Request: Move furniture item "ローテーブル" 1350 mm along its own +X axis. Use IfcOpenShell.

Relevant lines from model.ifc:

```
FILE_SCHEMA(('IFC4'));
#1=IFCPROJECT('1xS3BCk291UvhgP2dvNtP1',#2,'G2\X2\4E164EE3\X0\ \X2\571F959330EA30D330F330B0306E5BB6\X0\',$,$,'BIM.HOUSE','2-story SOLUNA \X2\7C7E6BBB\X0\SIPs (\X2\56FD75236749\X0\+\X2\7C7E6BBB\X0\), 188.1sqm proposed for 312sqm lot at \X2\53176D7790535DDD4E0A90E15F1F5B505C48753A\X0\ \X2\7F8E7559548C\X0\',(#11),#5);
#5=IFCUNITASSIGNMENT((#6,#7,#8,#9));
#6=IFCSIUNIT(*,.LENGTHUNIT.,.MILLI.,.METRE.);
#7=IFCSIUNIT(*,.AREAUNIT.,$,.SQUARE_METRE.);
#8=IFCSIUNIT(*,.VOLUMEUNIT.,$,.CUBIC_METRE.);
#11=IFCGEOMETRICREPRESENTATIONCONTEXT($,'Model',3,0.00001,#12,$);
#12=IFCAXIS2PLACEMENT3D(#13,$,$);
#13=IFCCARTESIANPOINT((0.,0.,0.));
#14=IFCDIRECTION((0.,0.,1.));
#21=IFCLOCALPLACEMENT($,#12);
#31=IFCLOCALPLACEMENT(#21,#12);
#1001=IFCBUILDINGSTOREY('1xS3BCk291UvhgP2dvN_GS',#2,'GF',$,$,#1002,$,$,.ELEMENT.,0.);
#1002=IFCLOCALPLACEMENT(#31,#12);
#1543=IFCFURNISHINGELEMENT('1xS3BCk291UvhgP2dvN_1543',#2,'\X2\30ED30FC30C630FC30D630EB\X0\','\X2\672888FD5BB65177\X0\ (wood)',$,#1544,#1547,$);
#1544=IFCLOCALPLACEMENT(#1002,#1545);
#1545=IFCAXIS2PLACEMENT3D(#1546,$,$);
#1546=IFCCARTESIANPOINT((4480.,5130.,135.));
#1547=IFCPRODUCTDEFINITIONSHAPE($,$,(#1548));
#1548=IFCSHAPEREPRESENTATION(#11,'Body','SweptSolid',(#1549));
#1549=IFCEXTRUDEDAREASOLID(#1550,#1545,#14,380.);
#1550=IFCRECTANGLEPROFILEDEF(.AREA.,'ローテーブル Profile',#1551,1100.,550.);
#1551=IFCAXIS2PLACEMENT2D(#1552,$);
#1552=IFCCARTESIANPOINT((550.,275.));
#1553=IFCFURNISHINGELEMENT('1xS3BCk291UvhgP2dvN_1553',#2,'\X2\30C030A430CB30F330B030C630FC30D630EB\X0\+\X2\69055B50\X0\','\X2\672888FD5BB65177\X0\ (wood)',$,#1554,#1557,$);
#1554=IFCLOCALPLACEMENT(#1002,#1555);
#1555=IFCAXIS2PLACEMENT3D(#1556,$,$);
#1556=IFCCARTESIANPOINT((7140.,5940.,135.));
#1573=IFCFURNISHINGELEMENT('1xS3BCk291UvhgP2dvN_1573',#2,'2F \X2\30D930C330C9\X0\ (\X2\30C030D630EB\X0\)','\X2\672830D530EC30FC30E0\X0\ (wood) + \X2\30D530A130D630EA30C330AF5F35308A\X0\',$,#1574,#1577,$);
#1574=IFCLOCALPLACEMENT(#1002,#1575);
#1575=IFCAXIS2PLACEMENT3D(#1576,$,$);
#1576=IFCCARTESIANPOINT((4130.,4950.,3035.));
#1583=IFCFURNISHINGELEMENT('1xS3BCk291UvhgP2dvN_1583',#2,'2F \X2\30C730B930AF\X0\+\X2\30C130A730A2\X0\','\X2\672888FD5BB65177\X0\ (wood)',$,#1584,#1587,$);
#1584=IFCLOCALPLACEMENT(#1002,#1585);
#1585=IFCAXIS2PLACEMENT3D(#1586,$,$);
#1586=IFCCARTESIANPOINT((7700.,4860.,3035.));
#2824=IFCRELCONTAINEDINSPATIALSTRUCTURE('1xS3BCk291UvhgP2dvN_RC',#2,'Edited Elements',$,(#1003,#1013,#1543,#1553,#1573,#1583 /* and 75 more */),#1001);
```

```python
import ifcopenshell
import ifcopenshell.api.geometry
import ifcopenshell.util.placement

model = ifcopenshell.open("model.ifc")

item = model.by_guid("1xS3BCk291UvhgP2dvN_1543")
matrix = ifcopenshell.util.placement.get_local_placement(item.ObjectPlacement)
matrix[:3, 3] += matrix[:3, 0] * 1350.0
ifcopenshell.api.geometry.edit_object_placement(model, product=item, matrix=matrix, is_si=False)

print(ifcopenshell.util.placement.get_local_placement(item.ObjectPlacement).round(3) + 0.0)

model.write("model_rev.ifc")
```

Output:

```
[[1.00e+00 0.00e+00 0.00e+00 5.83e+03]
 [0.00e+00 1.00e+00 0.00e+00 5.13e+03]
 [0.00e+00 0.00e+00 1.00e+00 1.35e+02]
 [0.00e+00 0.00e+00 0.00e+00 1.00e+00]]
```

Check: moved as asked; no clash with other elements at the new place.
